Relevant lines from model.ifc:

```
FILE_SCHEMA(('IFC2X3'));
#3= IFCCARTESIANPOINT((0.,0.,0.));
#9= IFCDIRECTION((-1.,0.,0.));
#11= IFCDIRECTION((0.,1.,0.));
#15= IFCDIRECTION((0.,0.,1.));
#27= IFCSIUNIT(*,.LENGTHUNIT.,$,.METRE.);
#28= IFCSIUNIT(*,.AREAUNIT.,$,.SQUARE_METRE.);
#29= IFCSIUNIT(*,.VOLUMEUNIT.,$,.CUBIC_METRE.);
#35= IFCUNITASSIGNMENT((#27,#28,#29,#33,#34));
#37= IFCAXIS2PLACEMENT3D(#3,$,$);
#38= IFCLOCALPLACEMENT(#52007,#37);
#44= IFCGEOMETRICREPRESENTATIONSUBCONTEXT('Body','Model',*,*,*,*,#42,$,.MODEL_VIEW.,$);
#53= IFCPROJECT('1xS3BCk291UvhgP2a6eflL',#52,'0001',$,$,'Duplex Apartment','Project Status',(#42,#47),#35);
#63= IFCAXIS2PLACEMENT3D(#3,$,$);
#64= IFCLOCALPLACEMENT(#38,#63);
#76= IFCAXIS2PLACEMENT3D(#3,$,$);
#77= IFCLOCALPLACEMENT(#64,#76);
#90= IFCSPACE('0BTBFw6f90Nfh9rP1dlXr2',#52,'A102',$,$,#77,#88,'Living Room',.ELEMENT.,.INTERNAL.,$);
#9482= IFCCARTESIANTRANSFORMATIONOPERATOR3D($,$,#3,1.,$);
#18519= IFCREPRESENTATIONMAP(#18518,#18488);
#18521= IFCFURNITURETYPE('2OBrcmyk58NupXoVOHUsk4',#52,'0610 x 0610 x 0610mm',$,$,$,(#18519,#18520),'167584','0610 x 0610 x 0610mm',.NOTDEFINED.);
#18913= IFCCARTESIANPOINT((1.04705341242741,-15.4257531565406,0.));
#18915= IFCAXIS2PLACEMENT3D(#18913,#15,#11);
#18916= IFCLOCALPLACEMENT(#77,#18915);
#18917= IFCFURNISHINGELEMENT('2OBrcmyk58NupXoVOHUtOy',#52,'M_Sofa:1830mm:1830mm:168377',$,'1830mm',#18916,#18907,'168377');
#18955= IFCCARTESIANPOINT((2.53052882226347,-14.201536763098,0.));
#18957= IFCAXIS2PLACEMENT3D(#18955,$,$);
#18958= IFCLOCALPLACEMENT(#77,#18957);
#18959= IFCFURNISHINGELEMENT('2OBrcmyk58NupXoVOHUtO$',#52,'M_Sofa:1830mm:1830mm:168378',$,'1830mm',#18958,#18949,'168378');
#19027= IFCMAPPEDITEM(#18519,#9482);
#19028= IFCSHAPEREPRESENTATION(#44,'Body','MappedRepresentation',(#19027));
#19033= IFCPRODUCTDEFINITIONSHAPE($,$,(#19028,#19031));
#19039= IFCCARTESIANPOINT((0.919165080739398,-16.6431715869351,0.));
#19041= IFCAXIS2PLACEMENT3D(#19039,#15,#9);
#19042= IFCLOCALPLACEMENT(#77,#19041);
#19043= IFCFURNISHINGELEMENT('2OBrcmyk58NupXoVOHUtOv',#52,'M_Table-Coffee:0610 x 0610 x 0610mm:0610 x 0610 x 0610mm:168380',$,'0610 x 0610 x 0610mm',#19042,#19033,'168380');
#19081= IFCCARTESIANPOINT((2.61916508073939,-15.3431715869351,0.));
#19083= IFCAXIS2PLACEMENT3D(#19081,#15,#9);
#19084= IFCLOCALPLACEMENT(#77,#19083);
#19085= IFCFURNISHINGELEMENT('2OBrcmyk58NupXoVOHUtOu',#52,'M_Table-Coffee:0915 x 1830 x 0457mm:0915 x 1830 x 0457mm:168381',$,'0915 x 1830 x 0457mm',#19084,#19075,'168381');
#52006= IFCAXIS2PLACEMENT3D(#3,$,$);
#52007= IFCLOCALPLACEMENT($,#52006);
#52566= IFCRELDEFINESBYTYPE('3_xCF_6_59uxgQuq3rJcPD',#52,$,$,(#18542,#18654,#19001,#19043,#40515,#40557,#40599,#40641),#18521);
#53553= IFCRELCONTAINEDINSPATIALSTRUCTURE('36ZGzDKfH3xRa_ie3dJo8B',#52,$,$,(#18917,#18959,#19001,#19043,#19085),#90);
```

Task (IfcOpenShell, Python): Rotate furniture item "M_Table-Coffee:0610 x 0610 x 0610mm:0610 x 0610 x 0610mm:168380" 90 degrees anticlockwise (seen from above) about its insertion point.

```python
import ifcopenshell
import ifcopenshell.api.geometry
import ifcopenshell.util.placement

model = ifcopenshell.open("model.ifc")

item = model.by_guid("2OBrcmyk58NupXoVOHUtOv")
matrix = ifcopenshell.util.placement.get_local_placement(item.ObjectPlacement)
matrix = matrix @ ifcopenshell.util.placement.rotation(90, "Z")
ifcopenshell.api.geometry.edit_object_placement(model, product=item, matrix=matrix, is_si=False)

print(ifcopenshell.util.placement.get_local_placement(item.ObjectPlacement).round(3) + 0.0)

model.write("model_edited.ifc")
```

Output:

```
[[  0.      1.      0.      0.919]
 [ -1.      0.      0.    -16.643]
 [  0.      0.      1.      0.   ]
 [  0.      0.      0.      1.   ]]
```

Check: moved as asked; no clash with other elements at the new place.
